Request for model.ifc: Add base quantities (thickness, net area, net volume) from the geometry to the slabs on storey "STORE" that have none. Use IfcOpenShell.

First a look at what the model holds.

```python
import ifcopenshell
import ifcopenshell.util.element
import ifcopenshell.util.unit

model = ifcopenshell.open("model.ifc")
print(model.schema)
for unit_type in ("LENGTHUNIT", "AREAUNIT", "VOLUMEUNIT"):
    print(unit_type, ifcopenshell.util.unit.calculate_unit_scale(model, unit_type))
storey = next(s for s in model.by_type("IfcBuildingStorey") if s.Name == "STORE")
slabs = [e for e in ifcopenshell.util.element.get_decomposition(storey) if e.is_a("IfcSlab")]
for e in sorted(slabs, key=lambda e: e.id()):
    print(e.id(), e.is_a(), e.Name, list(ifcopenshell.util.element.get_psets(e, qtos_only=True)), sep=" | ")
```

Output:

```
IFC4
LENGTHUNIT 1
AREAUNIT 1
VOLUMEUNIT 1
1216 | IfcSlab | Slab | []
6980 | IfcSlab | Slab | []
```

```python
import ifcopenshell
import ifcopenshell.api.pset
import ifcopenshell.geom
import ifcopenshell.util.element
import ifcopenshell.util.shape
import ifcopenshell.util.unit

model = ifcopenshell.open("model.ifc")
unit_scale = ifcopenshell.util.unit.calculate_unit_scale(model)
area_scale = ifcopenshell.util.unit.calculate_unit_scale(model, "AREAUNIT")
volume_scale = ifcopenshell.util.unit.calculate_unit_scale(model, "VOLUMEUNIT")
settings = ifcopenshell.geom.settings()

storey = next(s for s in model.by_type("IfcBuildingStorey") if s.Name == "STORE")
slabs = [e for e in ifcopenshell.util.element.get_decomposition(storey) if e.is_a("IfcSlab")]

for e in sorted(slabs, key=lambda e: e.id()):
    if ifcopenshell.util.element.get_psets(e, qtos_only=True, should_inherit=False):
        continue
    # Geometry comes back in metres, in the element's own axes.
    shape = ifcopenshell.geom.create_shape(settings, e)
    values = {
        "Width": ifcopenshell.util.shape.get_z(shape.geometry) / unit_scale,
        "NetArea": ifcopenshell.util.shape.get_footprint_area(shape.geometry) / area_scale,
        "NetVolume": ifcopenshell.util.shape.get_volume(shape.geometry) / volume_scale,
    }
    qto = ifcopenshell.api.pset.add_qto(model, product=e, name="Qto_SlabBaseQuantities")
    ifcopenshell.api.pset.edit_qto(model, qto=qto, properties=values)
    print(e.id(), {k: round(v, 3) for k, v in values.items()})

model.write("model_v2.ifc")
```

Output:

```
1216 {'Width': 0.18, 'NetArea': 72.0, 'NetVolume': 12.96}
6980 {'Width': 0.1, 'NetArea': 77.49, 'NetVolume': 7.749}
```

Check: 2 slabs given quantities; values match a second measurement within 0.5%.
